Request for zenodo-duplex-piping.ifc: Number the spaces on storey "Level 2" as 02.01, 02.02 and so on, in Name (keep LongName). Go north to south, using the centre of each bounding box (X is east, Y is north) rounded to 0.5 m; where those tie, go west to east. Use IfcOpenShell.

First a look at what the model holds.

```python
import ifcopenshell
import ifcopenshell.util.element
import ifcopenshell.util.placement

model = ifcopenshell.open("zenodo-duplex-piping.ifc")
print(model.schema)
storey = next(s for s in model.by_type("IfcBuildingStorey") if s.Name == "Level 2")
spaces = [e for e in ifcopenshell.util.element.get_decomposition(storey) if e.is_a("IfcSpace")]
for e in sorted(spaces, key=lambda e: e.id()):
    origin = ifcopenshell.util.placement.get_local_placement(e.ObjectPlacement)[:3, 3]
    print(e.id(), e.Name, e.LongName, origin.round(2) + 0.0, sep=" | ")
```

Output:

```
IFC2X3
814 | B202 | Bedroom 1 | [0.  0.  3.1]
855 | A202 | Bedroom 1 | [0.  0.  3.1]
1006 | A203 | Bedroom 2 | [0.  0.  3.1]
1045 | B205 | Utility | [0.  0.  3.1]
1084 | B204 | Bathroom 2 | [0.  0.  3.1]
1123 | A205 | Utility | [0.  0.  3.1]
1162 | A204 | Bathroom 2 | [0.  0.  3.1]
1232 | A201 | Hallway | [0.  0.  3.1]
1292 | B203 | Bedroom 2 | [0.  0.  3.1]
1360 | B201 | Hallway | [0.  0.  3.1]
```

```python
import ifcopenshell
import ifcopenshell.geom
import ifcopenshell.util.element
import ifcopenshell.util.shape

model = ifcopenshell.open("zenodo-duplex-piping.ifc")
settings = ifcopenshell.geom.settings()
settings.set("use-world-coords", True)


def centre(element):
    shape = ifcopenshell.geom.create_shape(settings, element)
    return ifcopenshell.util.shape.get_bbox_centroid(shape.geometry)


storey = next(s for s in model.by_type("IfcBuildingStorey") if s.Name == "Level 2")
spaces = [e for e in ifcopenshell.util.element.get_decomposition(storey) if e.is_a("IfcSpace")]

# Insertion points can sit at a corner or the storey origin, so sort by the geometry (in metres).
centres = {e: centre(e) for e in spaces}
spaces.sort(key=lambda e: (-round(centres[e][1] / 0.5), centres[e][0]))

for i, e in enumerate(spaces, start=1):
    number = f"02.{i:02d}"
    e.Name = number
    print(e.id(), number)

model.write("zenodo-duplex-piping_rev.ifc")
```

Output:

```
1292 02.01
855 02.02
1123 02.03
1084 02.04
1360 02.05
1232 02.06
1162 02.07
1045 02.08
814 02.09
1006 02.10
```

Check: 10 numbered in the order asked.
